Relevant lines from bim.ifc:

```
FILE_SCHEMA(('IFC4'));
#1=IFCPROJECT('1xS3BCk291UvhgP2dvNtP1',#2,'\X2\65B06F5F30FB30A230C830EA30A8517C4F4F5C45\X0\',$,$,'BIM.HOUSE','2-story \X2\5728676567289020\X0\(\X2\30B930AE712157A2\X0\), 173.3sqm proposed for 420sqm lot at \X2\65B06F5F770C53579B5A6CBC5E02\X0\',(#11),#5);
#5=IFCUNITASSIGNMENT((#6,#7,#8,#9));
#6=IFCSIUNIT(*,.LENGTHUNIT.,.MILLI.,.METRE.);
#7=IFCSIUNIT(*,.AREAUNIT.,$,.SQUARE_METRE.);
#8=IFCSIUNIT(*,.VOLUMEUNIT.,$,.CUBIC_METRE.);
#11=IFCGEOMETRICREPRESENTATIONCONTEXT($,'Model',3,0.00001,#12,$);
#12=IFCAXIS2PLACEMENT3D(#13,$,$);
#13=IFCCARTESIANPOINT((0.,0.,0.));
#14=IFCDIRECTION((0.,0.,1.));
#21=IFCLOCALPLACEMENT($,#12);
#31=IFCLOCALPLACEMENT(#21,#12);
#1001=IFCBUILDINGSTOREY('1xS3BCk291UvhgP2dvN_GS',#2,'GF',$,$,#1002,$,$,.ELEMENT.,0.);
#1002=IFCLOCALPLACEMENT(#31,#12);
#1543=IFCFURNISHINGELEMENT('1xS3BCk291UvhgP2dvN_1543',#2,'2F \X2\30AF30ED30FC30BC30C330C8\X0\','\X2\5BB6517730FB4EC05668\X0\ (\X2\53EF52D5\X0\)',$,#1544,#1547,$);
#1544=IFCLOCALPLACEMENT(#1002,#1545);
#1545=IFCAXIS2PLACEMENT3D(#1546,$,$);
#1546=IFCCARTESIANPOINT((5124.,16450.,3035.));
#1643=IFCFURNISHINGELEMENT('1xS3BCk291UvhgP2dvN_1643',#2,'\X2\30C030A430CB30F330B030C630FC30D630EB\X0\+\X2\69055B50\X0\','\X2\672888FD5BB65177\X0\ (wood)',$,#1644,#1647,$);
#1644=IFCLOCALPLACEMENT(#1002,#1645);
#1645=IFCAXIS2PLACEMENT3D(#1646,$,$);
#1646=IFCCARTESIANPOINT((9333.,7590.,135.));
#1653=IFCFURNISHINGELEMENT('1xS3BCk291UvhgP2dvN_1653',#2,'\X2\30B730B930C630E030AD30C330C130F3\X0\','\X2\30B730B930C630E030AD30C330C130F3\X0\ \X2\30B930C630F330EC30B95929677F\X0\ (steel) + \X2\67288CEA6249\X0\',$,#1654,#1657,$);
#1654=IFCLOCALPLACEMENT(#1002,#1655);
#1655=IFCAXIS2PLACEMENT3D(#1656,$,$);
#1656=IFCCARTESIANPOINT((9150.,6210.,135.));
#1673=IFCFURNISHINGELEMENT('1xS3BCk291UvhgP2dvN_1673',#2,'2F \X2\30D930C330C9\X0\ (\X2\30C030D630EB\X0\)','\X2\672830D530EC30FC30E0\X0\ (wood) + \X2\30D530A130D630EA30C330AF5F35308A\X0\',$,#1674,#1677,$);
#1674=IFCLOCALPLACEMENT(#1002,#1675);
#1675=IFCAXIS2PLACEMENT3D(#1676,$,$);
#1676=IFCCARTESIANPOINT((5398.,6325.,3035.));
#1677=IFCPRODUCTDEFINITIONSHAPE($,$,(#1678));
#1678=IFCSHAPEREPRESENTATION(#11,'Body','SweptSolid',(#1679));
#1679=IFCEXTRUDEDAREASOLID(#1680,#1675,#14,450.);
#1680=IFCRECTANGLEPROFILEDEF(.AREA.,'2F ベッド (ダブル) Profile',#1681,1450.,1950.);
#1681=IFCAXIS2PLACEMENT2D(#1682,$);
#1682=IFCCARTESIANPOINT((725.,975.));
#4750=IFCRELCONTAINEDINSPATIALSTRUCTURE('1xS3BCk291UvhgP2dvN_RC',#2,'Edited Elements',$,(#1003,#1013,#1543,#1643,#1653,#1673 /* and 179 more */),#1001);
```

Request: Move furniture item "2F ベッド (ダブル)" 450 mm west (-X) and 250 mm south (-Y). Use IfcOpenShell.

```python
import ifcopenshell
import ifcopenshell.api.geometry
import ifcopenshell.util.placement

model = ifcopenshell.open("bim.ifc")

item = model.by_guid("1xS3BCk291UvhgP2dvN_1673")
matrix = ifcopenshell.util.placement.get_local_placement(item.ObjectPlacement)
matrix[0, 3] -= 450.0
matrix[1, 3] -= 250.0
ifcopenshell.api.geometry.edit_object_placement(model, product=item, matrix=matrix, is_si=False)

print(ifcopenshell.util.placement.get_local_placement(item.ObjectPlacement).round(3) + 0.0)

model.write("bim-out.ifc")
```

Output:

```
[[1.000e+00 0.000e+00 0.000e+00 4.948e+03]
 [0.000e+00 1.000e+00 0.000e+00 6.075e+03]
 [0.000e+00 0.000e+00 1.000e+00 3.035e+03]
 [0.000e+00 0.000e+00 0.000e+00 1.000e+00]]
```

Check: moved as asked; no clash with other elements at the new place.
